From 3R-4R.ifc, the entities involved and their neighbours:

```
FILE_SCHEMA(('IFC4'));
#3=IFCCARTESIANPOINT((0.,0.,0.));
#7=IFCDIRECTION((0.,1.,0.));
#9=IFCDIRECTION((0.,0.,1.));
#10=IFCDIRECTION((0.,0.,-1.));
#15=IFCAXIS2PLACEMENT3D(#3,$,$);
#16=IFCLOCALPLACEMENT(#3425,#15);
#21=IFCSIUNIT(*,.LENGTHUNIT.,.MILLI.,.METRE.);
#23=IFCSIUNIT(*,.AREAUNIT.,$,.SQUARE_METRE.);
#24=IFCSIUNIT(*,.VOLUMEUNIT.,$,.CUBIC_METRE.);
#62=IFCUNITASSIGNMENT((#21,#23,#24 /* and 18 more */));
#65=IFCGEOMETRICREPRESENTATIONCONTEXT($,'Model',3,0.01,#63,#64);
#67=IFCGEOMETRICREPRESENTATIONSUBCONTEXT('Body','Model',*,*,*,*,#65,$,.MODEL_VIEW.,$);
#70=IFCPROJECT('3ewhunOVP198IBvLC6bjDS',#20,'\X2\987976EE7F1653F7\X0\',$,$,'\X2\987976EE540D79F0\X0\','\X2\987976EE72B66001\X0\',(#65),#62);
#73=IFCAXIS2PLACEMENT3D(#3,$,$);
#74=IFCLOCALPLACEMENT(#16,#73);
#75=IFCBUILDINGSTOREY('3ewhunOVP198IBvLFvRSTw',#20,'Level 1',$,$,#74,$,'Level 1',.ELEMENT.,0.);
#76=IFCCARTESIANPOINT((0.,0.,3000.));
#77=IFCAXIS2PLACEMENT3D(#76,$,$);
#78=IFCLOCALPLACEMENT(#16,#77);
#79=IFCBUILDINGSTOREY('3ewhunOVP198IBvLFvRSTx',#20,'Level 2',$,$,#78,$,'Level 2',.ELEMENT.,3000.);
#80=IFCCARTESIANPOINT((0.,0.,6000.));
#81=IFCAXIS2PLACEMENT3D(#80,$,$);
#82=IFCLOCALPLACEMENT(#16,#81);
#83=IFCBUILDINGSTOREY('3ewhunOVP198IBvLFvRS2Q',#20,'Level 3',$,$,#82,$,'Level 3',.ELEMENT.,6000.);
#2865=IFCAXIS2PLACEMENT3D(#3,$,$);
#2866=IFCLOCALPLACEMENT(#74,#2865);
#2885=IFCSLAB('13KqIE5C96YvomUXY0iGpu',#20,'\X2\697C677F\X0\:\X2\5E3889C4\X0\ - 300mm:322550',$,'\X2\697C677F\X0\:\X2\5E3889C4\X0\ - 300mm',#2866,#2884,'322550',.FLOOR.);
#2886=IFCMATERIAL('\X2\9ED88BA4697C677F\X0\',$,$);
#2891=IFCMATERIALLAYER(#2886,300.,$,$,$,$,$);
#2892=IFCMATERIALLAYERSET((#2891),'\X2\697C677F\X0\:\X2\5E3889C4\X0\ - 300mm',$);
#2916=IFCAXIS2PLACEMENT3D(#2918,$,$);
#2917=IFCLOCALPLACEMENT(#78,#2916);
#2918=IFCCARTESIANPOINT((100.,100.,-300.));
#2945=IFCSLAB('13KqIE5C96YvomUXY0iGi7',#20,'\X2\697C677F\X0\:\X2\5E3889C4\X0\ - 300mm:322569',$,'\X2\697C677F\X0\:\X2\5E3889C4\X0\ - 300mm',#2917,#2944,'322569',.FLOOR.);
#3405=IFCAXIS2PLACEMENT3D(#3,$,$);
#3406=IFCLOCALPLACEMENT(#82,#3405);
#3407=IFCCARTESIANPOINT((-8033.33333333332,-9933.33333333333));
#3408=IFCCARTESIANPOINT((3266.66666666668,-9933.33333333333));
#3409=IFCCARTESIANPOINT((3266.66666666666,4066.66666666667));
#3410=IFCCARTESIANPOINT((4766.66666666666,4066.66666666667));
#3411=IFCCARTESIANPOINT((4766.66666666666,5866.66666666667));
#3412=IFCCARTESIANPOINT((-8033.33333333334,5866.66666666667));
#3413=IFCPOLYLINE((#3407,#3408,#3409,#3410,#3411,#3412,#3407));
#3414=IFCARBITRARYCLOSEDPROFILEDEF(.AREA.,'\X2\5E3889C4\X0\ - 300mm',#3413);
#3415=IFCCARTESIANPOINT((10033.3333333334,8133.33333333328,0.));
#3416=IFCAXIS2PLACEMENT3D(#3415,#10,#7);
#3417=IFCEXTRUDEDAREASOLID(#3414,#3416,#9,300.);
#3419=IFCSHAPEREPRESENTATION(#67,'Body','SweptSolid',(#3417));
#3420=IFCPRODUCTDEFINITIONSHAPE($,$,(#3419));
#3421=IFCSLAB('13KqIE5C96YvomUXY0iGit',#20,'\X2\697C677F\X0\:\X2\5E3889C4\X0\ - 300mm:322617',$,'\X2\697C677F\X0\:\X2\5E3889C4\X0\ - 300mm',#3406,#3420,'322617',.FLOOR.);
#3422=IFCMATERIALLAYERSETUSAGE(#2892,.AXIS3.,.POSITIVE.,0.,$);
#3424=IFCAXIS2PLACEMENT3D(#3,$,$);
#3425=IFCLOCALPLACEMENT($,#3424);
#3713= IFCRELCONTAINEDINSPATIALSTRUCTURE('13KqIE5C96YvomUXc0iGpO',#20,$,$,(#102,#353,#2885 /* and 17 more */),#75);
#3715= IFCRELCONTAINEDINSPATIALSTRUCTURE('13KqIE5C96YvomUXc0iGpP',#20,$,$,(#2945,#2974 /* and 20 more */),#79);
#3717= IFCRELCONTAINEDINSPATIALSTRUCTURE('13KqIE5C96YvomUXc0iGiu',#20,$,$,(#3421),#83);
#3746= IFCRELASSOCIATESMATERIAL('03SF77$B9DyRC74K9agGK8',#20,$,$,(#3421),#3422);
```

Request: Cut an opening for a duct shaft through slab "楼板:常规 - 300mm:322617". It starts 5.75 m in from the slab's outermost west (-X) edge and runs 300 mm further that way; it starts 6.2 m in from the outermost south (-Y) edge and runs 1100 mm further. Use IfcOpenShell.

```python
import numpy as np
import ifcopenshell
import ifcopenshell.api.feature
import ifcopenshell.api.geometry
import ifcopenshell.api.root
import ifcopenshell.geom
import ifcopenshell.util.placement
import ifcopenshell.util.representation
import ifcopenshell.util.shape
import ifcopenshell.util.unit

model = ifcopenshell.open("3R-4R.ifc")
unit_scale = ifcopenshell.util.unit.calculate_unit_scale(model)
settings = ifcopenshell.geom.settings()


def volume(element):
    """Net volume in cubic metres, openings subtracted."""
    shape = ifcopenshell.geom.create_shape(settings, element)
    return ifcopenshell.util.shape.get_volume(shape.geometry)


slab = model.by_guid("13KqIE5C96YvomUXY0iGit")
before = volume(slab)

# Extent in the slab's own axes, in metres. The edges named are its -X and -Y sides.
slab_shape = ifcopenshell.geom.create_shape(settings, slab)
vertices = ifcopenshell.util.shape.get_vertices(slab_shape.geometry)
x_min, y_min, bottom = vertices.min(axis=0)
top = vertices[:, 2].max()

opening = ifcopenshell.api.root.create_entity(model, ifc_class="IfcOpeningElement", name="Duct shaft opening", predefined_type="OPENING")
context = ifcopenshell.util.representation.get_context(model, "Model", "Body", "MODEL_VIEW")
width, depth = 0.3, 1.1
outline = [(0.0, 0.0), (width, 0.0), (width, depth), (0.0, depth), (0.0, 0.0)]
# Overshoot both faces by 50 mm so the cut is clean.
shape = ifcopenshell.api.geometry.add_slab_representation(
    model, context=context, depth=top - bottom + 0.1, polyline=outline
)
ifcopenshell.api.geometry.assign_representation(model, product=opening, representation=shape)

matrix = ifcopenshell.util.placement.get_local_placement(slab.ObjectPlacement)
matrix[:, 3] = matrix @ np.append(np.array([x_min + 5.75, y_min + 6.2, bottom - 0.05]) / unit_scale, 1.0)
ifcopenshell.api.geometry.edit_object_placement(model, product=opening, matrix=matrix, is_si=False)
ifcopenshell.api.feature.add_feature(model, feature=opening, element=slab)

after = volume(slab)

print(f"slab volume {before:.3f} -> {after:.3f} m3")

model.write("3R-4R-out.ifc")
```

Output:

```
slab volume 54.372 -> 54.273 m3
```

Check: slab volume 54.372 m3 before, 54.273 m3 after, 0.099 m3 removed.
